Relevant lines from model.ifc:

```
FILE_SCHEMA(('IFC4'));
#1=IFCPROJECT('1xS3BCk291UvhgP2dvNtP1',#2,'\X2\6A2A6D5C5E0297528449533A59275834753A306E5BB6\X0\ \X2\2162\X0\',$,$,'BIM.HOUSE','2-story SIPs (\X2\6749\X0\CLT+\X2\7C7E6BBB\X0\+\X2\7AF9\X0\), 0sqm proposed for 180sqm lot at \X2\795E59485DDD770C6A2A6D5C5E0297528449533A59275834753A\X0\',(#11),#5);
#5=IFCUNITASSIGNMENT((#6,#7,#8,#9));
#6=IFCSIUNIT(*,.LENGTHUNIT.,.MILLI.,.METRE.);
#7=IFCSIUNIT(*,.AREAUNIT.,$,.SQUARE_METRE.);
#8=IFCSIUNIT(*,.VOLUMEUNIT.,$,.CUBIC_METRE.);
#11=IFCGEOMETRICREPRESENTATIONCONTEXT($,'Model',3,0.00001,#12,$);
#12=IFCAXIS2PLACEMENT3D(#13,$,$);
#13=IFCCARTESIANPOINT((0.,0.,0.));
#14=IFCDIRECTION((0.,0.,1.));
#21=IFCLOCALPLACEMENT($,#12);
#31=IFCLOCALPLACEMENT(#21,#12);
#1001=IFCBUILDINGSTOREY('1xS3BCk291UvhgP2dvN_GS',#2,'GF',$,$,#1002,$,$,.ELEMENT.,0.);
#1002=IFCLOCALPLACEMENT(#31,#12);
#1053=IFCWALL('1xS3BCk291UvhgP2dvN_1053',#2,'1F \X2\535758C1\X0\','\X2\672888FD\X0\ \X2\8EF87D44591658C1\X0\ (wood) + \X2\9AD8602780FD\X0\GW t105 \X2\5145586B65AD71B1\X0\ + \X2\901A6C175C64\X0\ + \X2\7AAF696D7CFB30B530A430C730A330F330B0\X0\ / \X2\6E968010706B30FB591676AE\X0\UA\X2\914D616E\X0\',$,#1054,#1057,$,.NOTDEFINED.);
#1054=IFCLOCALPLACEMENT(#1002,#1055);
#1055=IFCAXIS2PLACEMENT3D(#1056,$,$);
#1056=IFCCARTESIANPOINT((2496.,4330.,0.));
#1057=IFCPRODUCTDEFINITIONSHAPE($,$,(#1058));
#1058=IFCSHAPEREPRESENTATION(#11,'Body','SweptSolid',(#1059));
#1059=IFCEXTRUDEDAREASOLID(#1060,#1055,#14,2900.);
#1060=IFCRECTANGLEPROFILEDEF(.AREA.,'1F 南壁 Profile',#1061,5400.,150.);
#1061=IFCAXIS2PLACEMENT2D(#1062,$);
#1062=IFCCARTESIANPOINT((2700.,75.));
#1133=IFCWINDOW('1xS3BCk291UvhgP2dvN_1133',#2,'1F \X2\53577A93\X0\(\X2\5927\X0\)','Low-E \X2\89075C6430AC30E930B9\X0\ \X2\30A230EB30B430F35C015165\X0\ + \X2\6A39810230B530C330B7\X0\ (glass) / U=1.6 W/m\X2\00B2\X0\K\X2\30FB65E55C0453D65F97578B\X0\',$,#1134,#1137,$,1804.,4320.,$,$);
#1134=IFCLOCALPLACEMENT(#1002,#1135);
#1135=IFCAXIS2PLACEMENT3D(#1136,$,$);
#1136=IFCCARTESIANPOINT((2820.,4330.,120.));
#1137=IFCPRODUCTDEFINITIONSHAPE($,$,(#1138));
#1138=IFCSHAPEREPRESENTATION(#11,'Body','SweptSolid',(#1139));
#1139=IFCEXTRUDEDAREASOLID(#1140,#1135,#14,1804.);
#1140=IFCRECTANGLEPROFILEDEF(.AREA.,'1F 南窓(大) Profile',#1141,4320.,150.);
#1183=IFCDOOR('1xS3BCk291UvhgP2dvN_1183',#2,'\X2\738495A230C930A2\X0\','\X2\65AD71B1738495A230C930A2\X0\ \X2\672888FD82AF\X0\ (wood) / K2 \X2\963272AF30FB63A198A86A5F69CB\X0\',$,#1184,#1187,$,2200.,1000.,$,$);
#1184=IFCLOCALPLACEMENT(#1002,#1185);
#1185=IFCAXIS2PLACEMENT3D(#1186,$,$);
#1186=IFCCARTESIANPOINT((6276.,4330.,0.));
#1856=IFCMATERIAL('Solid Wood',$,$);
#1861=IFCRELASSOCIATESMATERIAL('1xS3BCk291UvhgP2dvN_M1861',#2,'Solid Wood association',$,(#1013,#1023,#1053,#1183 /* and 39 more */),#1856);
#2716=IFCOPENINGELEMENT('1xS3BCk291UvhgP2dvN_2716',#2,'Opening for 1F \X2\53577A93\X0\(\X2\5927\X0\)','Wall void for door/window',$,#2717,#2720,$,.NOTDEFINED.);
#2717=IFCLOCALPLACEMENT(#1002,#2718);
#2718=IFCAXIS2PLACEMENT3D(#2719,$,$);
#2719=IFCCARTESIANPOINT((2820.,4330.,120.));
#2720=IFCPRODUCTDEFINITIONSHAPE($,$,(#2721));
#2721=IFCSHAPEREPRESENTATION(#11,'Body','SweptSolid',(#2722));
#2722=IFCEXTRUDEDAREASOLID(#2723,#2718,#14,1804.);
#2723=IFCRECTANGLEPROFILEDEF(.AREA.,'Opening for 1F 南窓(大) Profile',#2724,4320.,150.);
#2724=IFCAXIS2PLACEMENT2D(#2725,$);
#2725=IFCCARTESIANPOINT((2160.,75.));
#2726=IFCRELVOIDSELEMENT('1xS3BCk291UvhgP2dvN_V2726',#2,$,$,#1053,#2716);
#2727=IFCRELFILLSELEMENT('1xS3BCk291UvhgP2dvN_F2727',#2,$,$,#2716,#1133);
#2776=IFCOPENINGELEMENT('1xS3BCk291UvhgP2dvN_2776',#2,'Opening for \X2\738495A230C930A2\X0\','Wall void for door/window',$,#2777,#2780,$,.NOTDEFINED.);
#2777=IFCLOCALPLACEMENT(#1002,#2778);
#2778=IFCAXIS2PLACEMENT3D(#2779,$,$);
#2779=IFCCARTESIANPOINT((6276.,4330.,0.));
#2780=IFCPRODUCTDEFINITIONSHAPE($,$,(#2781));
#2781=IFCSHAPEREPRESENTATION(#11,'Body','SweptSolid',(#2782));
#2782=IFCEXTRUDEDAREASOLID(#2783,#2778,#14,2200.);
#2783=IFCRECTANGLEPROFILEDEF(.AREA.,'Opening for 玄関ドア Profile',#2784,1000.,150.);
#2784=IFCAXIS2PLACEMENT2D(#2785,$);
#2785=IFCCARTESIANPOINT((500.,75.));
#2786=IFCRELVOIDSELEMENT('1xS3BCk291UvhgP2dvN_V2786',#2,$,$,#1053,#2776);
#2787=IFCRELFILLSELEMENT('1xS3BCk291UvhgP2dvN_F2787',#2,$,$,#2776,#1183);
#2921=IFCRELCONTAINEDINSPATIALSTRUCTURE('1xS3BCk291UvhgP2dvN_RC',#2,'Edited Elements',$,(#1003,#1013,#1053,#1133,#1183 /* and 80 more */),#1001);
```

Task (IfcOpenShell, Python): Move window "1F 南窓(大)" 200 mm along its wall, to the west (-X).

```python
import ifcopenshell
import ifcopenshell.api.geometry
import ifcopenshell.util.placement

model = ifcopenshell.open("model.ifc")

window = model.by_guid("1xS3BCk291UvhgP2dvN_1133")
opening = window.FillsVoids[0].RelatingOpeningElement
wall = opening.VoidsElements[0].RelatingBuildingElement

wall_matrix = ifcopenshell.util.placement.get_local_placement(wall.ObjectPlacement)
shift = wall_matrix[:3, 0] * -200.0
before = ifcopenshell.util.placement.get_local_placement(window.ObjectPlacement)[:3, 3].copy()

# The window is not placed relative to its opening, so move both.
for product in (opening, window):
    matrix = ifcopenshell.util.placement.get_local_placement(product.ObjectPlacement)
    matrix[:3, 3] += shift
    ifcopenshell.api.geometry.edit_object_placement(model, product=product, matrix=matrix, is_si=False)

after = ifcopenshell.util.placement.get_local_placement(window.ObjectPlacement)[:3, 3]
print("window moved by", (after - before).round(3) + 0.0)

model.write("model_updated.ifc")
```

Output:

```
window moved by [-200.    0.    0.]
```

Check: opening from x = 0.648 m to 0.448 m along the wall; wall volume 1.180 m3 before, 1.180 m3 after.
